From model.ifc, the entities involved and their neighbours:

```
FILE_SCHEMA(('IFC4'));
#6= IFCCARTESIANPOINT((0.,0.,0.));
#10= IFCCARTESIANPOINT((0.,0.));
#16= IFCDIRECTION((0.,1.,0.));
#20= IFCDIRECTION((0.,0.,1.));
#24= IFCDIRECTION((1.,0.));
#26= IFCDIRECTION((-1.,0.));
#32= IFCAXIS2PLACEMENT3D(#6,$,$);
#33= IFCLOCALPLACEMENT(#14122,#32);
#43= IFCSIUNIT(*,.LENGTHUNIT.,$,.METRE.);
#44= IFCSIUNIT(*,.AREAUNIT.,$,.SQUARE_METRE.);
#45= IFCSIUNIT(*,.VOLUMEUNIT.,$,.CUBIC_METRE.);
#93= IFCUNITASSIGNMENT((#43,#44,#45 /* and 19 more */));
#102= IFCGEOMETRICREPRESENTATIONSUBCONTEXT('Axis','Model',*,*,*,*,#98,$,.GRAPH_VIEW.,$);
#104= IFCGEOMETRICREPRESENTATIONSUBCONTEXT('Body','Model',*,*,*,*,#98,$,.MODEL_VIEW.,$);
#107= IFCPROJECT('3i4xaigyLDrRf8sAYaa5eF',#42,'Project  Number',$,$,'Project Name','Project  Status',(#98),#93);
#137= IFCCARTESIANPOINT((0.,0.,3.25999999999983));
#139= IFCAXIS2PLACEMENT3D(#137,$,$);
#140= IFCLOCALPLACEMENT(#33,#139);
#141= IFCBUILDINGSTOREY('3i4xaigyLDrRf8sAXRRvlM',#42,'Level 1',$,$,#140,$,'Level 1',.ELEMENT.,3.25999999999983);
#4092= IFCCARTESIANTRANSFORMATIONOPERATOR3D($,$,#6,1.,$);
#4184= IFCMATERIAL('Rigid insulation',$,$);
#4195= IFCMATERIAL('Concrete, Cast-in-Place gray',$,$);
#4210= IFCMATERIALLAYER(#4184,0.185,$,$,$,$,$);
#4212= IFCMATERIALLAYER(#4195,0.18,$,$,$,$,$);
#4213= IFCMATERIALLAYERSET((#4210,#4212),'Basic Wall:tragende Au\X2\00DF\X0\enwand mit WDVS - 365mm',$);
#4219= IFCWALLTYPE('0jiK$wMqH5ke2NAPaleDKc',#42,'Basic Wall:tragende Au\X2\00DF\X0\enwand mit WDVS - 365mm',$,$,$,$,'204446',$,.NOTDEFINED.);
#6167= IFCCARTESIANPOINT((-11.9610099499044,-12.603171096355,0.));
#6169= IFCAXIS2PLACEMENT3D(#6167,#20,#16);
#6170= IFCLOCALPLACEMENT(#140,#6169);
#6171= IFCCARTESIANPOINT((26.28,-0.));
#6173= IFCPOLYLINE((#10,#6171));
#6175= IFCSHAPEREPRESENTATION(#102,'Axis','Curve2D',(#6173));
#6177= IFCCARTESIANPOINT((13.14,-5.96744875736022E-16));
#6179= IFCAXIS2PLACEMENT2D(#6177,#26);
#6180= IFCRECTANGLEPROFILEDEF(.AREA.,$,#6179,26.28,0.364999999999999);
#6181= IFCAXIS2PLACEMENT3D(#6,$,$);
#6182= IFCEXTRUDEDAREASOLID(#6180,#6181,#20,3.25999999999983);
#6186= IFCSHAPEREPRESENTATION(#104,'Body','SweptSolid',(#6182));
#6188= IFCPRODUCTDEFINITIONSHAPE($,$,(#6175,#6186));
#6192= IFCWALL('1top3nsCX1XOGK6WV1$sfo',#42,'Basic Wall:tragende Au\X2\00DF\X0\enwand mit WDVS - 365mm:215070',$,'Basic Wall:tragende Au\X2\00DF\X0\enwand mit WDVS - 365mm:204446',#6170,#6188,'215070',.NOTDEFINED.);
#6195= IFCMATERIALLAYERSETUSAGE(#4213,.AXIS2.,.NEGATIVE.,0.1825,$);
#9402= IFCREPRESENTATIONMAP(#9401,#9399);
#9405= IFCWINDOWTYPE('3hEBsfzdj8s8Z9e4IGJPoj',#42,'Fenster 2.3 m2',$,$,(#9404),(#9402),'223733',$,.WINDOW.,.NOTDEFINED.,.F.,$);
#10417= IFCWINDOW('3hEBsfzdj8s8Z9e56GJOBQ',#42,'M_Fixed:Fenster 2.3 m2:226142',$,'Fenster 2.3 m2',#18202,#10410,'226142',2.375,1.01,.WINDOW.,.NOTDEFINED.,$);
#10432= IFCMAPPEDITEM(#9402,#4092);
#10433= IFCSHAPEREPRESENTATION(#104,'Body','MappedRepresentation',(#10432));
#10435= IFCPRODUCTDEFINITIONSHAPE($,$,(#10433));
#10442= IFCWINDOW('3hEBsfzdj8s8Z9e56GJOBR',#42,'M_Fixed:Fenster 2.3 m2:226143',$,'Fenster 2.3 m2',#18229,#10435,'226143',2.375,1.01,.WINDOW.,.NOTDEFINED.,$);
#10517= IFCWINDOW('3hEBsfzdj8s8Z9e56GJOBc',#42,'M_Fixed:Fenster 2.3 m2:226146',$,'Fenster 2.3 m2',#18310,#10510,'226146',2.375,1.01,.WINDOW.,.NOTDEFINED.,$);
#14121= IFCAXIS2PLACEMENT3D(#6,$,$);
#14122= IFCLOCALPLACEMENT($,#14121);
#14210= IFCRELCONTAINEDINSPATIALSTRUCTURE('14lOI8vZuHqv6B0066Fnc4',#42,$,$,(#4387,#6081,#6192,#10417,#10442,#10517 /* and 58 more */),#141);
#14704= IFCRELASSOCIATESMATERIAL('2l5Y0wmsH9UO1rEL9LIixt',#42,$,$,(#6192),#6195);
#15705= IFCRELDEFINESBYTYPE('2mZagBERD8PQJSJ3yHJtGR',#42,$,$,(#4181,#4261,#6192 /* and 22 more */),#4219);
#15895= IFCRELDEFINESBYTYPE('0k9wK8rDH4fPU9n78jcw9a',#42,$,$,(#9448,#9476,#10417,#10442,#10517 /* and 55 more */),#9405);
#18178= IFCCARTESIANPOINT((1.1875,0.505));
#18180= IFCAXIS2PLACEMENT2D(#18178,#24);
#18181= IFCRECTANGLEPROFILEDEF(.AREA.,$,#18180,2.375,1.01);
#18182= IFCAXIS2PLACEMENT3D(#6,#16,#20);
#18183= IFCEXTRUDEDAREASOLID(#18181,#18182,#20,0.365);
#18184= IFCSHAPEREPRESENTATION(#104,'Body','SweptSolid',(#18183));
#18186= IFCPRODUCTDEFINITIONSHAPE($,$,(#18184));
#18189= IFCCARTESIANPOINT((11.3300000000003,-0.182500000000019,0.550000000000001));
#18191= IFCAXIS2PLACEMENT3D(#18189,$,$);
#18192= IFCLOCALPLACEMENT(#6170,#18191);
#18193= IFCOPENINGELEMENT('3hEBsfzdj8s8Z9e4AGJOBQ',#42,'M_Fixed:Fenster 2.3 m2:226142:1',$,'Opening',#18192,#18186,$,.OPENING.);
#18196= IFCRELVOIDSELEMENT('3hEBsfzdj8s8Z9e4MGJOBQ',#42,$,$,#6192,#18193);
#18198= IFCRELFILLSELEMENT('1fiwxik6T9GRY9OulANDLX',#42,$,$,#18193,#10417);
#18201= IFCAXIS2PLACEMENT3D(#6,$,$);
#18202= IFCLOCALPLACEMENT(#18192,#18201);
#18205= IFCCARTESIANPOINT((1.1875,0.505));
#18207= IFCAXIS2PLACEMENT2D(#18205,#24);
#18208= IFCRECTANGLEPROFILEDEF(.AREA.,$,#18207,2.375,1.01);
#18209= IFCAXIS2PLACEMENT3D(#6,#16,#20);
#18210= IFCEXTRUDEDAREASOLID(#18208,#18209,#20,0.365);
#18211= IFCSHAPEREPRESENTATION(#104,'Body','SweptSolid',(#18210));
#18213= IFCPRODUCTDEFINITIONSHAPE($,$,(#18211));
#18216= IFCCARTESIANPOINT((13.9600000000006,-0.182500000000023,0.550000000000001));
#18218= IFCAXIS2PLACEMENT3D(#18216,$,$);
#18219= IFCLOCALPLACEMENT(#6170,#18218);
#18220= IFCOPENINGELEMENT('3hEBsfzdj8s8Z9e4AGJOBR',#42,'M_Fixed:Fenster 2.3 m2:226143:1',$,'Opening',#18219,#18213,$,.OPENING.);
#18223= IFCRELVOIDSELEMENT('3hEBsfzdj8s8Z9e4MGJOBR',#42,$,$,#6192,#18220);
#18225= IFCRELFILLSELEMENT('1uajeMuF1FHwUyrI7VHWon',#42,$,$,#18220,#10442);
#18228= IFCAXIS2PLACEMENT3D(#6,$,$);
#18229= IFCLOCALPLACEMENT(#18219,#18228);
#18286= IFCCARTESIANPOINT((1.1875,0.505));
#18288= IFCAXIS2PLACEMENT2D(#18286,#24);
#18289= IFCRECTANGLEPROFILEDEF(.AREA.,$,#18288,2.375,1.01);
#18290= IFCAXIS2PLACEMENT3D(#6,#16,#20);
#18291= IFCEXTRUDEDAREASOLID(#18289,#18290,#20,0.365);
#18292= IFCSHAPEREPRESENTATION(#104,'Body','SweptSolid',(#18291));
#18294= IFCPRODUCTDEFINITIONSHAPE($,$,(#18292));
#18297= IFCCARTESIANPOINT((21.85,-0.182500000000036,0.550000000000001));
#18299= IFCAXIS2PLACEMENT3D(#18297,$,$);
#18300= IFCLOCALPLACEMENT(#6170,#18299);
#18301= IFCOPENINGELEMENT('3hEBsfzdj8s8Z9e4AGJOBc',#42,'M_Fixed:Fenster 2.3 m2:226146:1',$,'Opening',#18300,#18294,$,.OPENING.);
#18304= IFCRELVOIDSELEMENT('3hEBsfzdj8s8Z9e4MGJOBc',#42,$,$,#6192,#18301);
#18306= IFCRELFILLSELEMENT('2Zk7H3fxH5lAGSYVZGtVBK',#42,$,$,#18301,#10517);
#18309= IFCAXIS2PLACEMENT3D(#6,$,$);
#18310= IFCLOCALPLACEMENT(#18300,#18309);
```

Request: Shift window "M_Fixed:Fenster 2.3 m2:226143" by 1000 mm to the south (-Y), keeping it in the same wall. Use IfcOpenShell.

```python
import ifcopenshell
import ifcopenshell.api.geometry
import ifcopenshell.util.placement

model = ifcopenshell.open("model.ifc")

window = model.by_guid("3hEBsfzdj8s8Z9e56GJOBR")
opening = window.FillsVoids[0].RelatingOpeningElement
wall = opening.VoidsElements[0].RelatingBuildingElement

wall_matrix = ifcopenshell.util.placement.get_local_placement(wall.ObjectPlacement)
shift = wall_matrix[:3, 0] * -1.0
before = ifcopenshell.util.placement.get_local_placement(window.ObjectPlacement)[:3, 3].copy()

# The window is placed relative to its opening, so it follows when the opening moves.
matrix = ifcopenshell.util.placement.get_local_placement(opening.ObjectPlacement)
matrix[:3, 3] += shift
ifcopenshell.api.geometry.edit_object_placement(
    model, product=opening, matrix=matrix, is_si=False, should_transform_children=True
)

after = ifcopenshell.util.placement.get_local_placement(window.ObjectPlacement)[:3, 3]
print("window moved by", (after - before).round(3) + 0.0)

model.write("model-out.ifc")
```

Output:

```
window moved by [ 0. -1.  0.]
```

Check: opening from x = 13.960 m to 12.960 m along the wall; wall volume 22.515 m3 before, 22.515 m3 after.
